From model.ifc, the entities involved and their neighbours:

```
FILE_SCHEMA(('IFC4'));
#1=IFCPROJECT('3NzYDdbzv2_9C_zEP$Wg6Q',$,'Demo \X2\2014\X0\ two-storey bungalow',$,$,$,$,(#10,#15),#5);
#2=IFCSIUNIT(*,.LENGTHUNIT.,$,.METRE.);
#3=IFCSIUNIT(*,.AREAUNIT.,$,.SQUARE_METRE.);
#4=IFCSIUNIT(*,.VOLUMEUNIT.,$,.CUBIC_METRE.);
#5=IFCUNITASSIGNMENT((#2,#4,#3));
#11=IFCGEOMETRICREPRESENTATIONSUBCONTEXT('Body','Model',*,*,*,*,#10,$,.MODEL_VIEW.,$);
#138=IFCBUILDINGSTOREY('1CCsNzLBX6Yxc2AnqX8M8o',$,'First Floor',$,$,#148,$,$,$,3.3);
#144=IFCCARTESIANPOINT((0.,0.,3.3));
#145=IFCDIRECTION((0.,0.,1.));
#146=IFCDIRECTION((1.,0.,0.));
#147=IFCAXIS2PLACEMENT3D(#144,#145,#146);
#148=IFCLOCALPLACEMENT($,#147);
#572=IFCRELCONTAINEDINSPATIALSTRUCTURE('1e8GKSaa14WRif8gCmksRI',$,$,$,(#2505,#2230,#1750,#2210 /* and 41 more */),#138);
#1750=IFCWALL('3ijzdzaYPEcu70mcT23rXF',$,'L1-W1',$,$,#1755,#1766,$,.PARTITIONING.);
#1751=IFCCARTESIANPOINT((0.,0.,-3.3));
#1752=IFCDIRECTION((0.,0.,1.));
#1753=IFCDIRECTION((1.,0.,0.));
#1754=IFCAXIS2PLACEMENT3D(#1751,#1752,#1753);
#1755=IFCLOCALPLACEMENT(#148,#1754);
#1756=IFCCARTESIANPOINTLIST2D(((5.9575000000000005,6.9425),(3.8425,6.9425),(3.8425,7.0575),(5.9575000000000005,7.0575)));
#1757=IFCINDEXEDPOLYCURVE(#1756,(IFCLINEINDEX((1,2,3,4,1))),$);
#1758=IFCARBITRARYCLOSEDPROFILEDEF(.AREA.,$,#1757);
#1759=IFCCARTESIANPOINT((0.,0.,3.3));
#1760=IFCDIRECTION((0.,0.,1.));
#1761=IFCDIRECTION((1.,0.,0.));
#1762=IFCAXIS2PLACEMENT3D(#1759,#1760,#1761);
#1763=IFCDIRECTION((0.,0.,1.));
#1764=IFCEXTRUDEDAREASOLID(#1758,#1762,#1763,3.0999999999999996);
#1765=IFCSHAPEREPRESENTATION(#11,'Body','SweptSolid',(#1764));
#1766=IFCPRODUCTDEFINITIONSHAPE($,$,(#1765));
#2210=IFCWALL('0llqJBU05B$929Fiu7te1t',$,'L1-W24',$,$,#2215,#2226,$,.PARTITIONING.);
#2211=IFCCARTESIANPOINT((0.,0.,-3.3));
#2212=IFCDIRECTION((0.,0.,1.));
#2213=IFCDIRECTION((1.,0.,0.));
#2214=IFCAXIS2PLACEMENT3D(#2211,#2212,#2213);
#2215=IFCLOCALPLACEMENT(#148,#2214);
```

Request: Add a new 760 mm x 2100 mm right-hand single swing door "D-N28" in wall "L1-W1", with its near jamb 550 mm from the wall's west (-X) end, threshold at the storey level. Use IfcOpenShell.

```python
import numpy as np
import ifcopenshell
import ifcopenshell.api.feature
import ifcopenshell.api.geometry
import ifcopenshell.api.root
import ifcopenshell.api.spatial
import ifcopenshell.geom
import ifcopenshell.util.element
import ifcopenshell.util.placement
import ifcopenshell.util.representation
import ifcopenshell.util.shape
import ifcopenshell.util.unit

model = ifcopenshell.open("model.ifc")
unit_scale = ifcopenshell.util.unit.calculate_unit_scale(model)
settings = ifcopenshell.geom.settings()


def volume(element):
    """Net volume in cubic metres, openings subtracted."""
    shape = ifcopenshell.geom.create_shape(settings, element)
    return ifcopenshell.util.shape.get_volume(shape.geometry)


wall = model.by_guid("3ijzdzaYPEcu70mcT23rXF")
storey = ifcopenshell.util.element.get_container(wall, ifc_class="IfcBuildingStorey")
context = ifcopenshell.util.representation.get_context(model, "Model", "Body", "MODEL_VIEW")
before = volume(wall)

width, height, from_end, sill = 0.76, 2.1, 0.55, 0.0  # metres

# The wall runs along its own X axis, and the end named is its -X end.
wall_shape = ifcopenshell.geom.create_shape(settings, wall)
x, y, z = ifcopenshell.util.shape.get_vertices(wall_shape.geometry).T
start = x.min() + from_end
face, thickness = float(y.min()), float(y.max() - y.min())
wall_matrix = ifcopenshell.util.placement.get_local_placement(wall.ObjectPlacement)
level = ifcopenshell.util.placement.get_local_placement(storey.ObjectPlacement)[2, 3]


def in_wall(x, y):
    """Placement at x, y metres in the wall's axes, at sill height."""
    matrix = wall_matrix.copy()
    matrix[:, 3] = wall_matrix @ np.array([x / unit_scale, y / unit_scale, 0.0, 1.0])
    matrix[2, 3] = level + sill / unit_scale
    return matrix


# Opening: a box that overshoots both wall faces by 50 mm.
opening = ifcopenshell.api.root.create_entity(model, ifc_class="IfcOpeningElement", predefined_type="OPENING")
box = ifcopenshell.api.geometry.add_wall_representation(
    model, context=context, length=width, height=height, thickness=thickness + 0.1
)
ifcopenshell.api.geometry.assign_representation(model, product=opening, representation=box)
ifcopenshell.api.geometry.edit_object_placement(model, product=opening, matrix=in_wall(start, face - 0.05), is_si=False)
ifcopenshell.api.feature.add_feature(model, feature=opening, element=wall)

door = ifcopenshell.api.root.create_entity(model, ifc_class="IfcDoor", name="D-N28", predefined_type="DOOR")
door.OverallWidth, door.OverallHeight = width / unit_scale, height / unit_scale
door.OperationType = "SINGLE_SWING_RIGHT"
body = ifcopenshell.api.geometry.add_door_representation(
    model,
    context=context,
    overall_width=door.OverallWidth,
    overall_height=door.OverallHeight,
    operation_type="SINGLE_SWING_RIGHT",
    lining_properties={"LiningDepth": thickness / unit_scale, "ThresholdDepth": thickness / unit_scale},
)
ifcopenshell.api.geometry.assign_representation(model, product=door, representation=body)
ifcopenshell.api.spatial.assign_container(model, products=[door], relating_structure=storey)
ifcopenshell.api.feature.add_filling(model, opening=opening, element=door)

# The lining spans the wall, so the door starts at the wall face.
ifcopenshell.api.geometry.edit_object_placement(model, product=door, matrix=in_wall(start, face), is_si=False)

after = volume(wall)

print(f"wall volume {before:.3f} -> {after:.3f} m3")

model.write("model_edited.ifc")
```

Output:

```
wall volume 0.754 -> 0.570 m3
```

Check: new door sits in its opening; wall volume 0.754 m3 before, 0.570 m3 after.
